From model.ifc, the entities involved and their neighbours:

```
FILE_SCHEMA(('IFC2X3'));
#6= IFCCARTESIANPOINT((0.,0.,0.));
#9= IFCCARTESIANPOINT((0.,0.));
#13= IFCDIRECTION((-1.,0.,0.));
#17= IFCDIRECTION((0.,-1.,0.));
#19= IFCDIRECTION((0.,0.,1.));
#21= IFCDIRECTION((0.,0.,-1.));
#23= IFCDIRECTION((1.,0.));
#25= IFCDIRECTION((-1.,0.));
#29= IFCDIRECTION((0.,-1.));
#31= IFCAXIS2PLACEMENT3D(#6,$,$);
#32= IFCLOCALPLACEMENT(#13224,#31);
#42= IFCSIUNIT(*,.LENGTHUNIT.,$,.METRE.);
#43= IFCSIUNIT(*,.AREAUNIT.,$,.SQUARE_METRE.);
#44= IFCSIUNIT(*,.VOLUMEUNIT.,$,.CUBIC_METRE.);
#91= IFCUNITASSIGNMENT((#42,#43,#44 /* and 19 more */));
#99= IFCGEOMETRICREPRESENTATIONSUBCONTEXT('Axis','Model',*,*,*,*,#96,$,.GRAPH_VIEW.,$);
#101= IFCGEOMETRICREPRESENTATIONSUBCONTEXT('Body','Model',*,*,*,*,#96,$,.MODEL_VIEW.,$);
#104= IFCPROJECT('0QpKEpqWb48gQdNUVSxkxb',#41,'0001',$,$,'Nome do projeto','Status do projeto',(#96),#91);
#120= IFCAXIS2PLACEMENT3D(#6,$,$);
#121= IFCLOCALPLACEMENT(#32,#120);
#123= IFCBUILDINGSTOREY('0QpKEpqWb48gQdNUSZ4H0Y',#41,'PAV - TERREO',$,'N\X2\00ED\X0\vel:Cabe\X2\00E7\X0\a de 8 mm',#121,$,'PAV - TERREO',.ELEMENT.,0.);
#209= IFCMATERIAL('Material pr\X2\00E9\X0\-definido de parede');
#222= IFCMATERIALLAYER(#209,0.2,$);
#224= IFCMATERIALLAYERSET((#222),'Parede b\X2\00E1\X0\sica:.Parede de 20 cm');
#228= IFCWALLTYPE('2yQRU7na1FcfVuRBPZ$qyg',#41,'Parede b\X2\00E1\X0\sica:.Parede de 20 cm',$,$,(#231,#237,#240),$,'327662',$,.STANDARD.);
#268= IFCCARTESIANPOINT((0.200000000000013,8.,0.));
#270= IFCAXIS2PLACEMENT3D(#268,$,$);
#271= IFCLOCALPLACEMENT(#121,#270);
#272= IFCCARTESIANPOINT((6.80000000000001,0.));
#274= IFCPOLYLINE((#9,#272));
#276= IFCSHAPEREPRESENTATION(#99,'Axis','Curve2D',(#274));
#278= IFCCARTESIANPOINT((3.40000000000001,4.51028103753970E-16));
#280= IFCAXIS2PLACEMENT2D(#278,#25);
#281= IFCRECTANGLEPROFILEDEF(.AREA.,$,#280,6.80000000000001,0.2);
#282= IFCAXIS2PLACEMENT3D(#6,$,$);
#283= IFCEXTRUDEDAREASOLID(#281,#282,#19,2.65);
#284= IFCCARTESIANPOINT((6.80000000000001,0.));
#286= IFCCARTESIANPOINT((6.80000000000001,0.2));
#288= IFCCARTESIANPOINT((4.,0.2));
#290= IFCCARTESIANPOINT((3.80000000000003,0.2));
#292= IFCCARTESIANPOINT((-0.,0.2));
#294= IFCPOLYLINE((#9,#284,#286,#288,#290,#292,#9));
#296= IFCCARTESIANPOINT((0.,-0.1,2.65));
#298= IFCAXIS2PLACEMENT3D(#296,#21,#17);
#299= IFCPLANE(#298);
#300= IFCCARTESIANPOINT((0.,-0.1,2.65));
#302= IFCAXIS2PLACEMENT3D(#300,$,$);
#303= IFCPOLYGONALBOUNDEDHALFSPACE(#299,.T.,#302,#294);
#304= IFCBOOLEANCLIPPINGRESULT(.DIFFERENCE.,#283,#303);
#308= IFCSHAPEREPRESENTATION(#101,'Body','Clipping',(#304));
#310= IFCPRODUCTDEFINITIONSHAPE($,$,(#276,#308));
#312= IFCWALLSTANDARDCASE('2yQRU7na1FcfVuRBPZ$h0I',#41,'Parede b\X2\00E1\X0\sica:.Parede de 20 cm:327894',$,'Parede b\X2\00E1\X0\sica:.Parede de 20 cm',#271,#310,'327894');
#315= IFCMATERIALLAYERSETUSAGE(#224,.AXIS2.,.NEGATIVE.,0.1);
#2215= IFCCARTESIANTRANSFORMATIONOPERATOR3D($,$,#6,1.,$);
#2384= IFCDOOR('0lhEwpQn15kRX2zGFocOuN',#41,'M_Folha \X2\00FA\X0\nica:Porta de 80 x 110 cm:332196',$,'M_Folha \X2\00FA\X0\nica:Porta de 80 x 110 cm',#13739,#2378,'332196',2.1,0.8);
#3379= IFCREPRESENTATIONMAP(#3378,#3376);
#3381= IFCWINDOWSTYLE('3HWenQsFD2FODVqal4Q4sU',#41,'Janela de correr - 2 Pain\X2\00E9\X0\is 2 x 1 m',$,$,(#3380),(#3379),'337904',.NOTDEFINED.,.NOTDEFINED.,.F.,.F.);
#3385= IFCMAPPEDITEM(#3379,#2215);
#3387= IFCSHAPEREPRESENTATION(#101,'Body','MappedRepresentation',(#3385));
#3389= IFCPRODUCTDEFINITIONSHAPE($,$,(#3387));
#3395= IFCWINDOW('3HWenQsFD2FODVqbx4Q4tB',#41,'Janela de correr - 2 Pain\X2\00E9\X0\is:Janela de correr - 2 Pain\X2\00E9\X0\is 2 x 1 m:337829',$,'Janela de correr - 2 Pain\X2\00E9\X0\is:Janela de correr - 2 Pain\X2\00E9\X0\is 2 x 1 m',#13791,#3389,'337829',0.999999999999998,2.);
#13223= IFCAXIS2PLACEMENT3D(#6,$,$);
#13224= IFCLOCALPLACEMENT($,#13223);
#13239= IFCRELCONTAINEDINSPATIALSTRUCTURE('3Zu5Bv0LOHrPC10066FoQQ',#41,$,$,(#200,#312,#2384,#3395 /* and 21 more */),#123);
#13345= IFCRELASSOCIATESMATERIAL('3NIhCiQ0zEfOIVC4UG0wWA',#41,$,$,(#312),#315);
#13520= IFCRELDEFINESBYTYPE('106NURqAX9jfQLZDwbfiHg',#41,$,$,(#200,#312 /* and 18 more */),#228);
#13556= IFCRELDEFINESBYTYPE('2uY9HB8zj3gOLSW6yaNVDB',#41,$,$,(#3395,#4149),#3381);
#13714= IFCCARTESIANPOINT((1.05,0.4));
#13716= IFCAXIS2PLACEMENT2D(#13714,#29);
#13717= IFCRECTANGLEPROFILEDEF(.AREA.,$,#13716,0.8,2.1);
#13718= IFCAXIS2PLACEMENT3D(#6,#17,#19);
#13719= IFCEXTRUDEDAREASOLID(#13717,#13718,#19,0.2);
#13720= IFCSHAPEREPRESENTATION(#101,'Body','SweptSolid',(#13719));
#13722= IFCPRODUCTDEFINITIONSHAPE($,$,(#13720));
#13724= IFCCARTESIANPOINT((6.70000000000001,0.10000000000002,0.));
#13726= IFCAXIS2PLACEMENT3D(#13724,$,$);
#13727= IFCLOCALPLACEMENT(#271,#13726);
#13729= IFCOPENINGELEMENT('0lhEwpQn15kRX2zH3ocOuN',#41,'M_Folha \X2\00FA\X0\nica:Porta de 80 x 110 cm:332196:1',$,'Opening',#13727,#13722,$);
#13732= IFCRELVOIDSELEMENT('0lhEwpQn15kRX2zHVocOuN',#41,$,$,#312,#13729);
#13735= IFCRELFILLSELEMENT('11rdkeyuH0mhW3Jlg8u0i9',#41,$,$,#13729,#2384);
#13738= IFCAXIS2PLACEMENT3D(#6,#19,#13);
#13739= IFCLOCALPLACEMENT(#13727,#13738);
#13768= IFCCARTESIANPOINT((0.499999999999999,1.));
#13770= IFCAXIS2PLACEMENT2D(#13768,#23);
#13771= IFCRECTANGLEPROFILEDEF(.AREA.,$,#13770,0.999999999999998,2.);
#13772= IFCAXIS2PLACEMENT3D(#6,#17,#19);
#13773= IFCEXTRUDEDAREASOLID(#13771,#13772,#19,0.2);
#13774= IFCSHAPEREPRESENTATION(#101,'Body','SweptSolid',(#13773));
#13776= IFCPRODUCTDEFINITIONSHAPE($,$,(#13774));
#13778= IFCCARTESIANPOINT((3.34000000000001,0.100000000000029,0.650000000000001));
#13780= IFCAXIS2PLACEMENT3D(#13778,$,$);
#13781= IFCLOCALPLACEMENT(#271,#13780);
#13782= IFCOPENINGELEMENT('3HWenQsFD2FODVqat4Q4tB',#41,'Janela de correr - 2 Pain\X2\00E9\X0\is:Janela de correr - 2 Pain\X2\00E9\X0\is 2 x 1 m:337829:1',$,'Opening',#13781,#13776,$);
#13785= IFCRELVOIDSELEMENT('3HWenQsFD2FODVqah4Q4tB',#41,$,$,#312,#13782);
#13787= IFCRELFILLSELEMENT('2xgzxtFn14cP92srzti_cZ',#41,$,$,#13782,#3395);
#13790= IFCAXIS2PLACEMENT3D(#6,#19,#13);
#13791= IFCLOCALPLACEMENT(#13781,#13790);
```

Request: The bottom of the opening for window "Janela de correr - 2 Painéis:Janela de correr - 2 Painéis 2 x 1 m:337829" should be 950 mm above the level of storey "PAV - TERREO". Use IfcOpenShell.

```python
import numpy as np
import ifcopenshell
import ifcopenshell.api.geometry
import ifcopenshell.geom
import ifcopenshell.util.element
import ifcopenshell.util.placement
import ifcopenshell.util.shape
import ifcopenshell.util.unit

model = ifcopenshell.open("model.ifc")
unit_scale = ifcopenshell.util.unit.calculate_unit_scale(model)

window = model.by_id(3395)
opening = window.FillsVoids[0].RelatingOpeningElement
storey = ifcopenshell.util.element.get_container(window, ifc_class="IfcBuildingStorey")
level = ifcopenshell.util.placement.get_local_placement(storey.ObjectPlacement)[2, 3]

# The opening's origin need not be at the sill, so measure its lowest point.
shape = ifcopenshell.geom.create_shape(ifcopenshell.geom.settings(), opening)
bottom = ifcopenshell.util.shape.get_shape_bottom_elevation(shape, shape.geometry) / unit_scale
dz = level + 0.95 / unit_scale - bottom

shift = np.array([0.0, 0.0, dz])
# The window is placed relative to its opening, so it follows when the opening moves.
matrix = ifcopenshell.util.placement.get_local_placement(opening.ObjectPlacement)
matrix[:3, 3] += shift
ifcopenshell.api.geometry.edit_object_placement(
    model, product=opening, matrix=matrix, is_si=False, should_transform_children=True
)

print(f"moved by {dz * unit_scale:+.3f} m")

model.write("model_rev.ifc")
```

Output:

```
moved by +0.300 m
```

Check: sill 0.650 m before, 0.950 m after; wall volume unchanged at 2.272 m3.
